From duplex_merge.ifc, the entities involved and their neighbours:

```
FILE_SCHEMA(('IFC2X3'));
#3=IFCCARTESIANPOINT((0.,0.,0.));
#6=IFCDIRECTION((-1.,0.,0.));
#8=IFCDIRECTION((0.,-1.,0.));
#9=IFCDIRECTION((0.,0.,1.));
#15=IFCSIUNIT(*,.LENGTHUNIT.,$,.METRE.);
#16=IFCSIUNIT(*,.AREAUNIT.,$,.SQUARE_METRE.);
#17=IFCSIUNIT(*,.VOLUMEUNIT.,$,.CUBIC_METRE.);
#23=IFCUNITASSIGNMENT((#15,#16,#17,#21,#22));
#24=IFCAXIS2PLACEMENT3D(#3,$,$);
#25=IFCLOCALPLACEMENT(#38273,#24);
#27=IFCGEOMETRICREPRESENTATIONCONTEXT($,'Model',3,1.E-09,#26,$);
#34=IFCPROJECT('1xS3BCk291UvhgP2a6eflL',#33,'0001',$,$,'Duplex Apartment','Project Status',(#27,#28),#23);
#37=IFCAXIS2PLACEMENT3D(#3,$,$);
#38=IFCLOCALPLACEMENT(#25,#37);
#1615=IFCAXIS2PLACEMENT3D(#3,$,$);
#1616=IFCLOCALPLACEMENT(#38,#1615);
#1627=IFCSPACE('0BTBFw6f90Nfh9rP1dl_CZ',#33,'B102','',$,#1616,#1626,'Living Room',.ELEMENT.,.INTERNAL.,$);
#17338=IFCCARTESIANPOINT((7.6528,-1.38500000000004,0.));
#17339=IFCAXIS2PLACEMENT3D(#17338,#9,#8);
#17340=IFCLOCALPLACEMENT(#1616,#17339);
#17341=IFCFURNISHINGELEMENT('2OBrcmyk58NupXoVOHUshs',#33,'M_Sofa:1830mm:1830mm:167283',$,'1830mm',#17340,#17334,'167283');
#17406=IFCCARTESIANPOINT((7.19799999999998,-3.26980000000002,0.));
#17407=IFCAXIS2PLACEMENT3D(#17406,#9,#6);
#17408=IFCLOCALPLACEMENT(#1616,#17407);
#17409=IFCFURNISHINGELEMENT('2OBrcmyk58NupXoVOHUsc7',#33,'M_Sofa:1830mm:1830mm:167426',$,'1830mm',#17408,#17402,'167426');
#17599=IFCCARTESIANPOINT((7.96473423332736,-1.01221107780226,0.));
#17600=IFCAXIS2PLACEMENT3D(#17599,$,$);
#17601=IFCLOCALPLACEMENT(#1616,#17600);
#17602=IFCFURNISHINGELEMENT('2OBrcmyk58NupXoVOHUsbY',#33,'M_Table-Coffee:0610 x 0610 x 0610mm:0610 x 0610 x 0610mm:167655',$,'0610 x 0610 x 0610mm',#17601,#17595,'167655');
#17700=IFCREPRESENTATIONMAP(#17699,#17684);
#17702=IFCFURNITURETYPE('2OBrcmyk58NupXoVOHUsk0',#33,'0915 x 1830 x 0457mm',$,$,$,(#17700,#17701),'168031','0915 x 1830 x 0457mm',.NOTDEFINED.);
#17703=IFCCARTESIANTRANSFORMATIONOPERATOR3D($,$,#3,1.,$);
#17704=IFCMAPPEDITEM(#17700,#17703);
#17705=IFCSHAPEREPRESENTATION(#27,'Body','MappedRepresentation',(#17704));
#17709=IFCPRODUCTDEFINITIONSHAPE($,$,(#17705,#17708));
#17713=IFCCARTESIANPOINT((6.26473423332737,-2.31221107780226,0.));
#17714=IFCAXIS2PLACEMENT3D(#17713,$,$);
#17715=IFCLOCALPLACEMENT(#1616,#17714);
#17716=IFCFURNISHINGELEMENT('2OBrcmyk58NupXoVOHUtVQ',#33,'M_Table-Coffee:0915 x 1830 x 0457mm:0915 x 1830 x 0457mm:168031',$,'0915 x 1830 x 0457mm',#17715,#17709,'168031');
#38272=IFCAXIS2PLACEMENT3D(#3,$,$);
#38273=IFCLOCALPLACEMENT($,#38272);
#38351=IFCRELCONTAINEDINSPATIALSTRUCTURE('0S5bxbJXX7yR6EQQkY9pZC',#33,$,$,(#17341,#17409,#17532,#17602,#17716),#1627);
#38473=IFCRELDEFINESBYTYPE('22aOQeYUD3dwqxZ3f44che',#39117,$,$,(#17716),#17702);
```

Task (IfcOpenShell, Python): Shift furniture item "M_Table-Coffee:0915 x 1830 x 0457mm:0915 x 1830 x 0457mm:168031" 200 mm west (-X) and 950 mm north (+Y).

```python
import ifcopenshell
import ifcopenshell.api.geometry
import ifcopenshell.util.placement

model = ifcopenshell.open("duplex_merge.ifc")

item = model.by_guid("2OBrcmyk58NupXoVOHUtVQ")
matrix = ifcopenshell.util.placement.get_local_placement(item.ObjectPlacement)
matrix[0, 3] -= 0.2
matrix[1, 3] += 0.95
ifcopenshell.api.geometry.edit_object_placement(model, product=item, matrix=matrix, is_si=False)

print(ifcopenshell.util.placement.get_local_placement(item.ObjectPlacement).round(3) + 0.0)

model.write("duplex_merge-out.ifc")
```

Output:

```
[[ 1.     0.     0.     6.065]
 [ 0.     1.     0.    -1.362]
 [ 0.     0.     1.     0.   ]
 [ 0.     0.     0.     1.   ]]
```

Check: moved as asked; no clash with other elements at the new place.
